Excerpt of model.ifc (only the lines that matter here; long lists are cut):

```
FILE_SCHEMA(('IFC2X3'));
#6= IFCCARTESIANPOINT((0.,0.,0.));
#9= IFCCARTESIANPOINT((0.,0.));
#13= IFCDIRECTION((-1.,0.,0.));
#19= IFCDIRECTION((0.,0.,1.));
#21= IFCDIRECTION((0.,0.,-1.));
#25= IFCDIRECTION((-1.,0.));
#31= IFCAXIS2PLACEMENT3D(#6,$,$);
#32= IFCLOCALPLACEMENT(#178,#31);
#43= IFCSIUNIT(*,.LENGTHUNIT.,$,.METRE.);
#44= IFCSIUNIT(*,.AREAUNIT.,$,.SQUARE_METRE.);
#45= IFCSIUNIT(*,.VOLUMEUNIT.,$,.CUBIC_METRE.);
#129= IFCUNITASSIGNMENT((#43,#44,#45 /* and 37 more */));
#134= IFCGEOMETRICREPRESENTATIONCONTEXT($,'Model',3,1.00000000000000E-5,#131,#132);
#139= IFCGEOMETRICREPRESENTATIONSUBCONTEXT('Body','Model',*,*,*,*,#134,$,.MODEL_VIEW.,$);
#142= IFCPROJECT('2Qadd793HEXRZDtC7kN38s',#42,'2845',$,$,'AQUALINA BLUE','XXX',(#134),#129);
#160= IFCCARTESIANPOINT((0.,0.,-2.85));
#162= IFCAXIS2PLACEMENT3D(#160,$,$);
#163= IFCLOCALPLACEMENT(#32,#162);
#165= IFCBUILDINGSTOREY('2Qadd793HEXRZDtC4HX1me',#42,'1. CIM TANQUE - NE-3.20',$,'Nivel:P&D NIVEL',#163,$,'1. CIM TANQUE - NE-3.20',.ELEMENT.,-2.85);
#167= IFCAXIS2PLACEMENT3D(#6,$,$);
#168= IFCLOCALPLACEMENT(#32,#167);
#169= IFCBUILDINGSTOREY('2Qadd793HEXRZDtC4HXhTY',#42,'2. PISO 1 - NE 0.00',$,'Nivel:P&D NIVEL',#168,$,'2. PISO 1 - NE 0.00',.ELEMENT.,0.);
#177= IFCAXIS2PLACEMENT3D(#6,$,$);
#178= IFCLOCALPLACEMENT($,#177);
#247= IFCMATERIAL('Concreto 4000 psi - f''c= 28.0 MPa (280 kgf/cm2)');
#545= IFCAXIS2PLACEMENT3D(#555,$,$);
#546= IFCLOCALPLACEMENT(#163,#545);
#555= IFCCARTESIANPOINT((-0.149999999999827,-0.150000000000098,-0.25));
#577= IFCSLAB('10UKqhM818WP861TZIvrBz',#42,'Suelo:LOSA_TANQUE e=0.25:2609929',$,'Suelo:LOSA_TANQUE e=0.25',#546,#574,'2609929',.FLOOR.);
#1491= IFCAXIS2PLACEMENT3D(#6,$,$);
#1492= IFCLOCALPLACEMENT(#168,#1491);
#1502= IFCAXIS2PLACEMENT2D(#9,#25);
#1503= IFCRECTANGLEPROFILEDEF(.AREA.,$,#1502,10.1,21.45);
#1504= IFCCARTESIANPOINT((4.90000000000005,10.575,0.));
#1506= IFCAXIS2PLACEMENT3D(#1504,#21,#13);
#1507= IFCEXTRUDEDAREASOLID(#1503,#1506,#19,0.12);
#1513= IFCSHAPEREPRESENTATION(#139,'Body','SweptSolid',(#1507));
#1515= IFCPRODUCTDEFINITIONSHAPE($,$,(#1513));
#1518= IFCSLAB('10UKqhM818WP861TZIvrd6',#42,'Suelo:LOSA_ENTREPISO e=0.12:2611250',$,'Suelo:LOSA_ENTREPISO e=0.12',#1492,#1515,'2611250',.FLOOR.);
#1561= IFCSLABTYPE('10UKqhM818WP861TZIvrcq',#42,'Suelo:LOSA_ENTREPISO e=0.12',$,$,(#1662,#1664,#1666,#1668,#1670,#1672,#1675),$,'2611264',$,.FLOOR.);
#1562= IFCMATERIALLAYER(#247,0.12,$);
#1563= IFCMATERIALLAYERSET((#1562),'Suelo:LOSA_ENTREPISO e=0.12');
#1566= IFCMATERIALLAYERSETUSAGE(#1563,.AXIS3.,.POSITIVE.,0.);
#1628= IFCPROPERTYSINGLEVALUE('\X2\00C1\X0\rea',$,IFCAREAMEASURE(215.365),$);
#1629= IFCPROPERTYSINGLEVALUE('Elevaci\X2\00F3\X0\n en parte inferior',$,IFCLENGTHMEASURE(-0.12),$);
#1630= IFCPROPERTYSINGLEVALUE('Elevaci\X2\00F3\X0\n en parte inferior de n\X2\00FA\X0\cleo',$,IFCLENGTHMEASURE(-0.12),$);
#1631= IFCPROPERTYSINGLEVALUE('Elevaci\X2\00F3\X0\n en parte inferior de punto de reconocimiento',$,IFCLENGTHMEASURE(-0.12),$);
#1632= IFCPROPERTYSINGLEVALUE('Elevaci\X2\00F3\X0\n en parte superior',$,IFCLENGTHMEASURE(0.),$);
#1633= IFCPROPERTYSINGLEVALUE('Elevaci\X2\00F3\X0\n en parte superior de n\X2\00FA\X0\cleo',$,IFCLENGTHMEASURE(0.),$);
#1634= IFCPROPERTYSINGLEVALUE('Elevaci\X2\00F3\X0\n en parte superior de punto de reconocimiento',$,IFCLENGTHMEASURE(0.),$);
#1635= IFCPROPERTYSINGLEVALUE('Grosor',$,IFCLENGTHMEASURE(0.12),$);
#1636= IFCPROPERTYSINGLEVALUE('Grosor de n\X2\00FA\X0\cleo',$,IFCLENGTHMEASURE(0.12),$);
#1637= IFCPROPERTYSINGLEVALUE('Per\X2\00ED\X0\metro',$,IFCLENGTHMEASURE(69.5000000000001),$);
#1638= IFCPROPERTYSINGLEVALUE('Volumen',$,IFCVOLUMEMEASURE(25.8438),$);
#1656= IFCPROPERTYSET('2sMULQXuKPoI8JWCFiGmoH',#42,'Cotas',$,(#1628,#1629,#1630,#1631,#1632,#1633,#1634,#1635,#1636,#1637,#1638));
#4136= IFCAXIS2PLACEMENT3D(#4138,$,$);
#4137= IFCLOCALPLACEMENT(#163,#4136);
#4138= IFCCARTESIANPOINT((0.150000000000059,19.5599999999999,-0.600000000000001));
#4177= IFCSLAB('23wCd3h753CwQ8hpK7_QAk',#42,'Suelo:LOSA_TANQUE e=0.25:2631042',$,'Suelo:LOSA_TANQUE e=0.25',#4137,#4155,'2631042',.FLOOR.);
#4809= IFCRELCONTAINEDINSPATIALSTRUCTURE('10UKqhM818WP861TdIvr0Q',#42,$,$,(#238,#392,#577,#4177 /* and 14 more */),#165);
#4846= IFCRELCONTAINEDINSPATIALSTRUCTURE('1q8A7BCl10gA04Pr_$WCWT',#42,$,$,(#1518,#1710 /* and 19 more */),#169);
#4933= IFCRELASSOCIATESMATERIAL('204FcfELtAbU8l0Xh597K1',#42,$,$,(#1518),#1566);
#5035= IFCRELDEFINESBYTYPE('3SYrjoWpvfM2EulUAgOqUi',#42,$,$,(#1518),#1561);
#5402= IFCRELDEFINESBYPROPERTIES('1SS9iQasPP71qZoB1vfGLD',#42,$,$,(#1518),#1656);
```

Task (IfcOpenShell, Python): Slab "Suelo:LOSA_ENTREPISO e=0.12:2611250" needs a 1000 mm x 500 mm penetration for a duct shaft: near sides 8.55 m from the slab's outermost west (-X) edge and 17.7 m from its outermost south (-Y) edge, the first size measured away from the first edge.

```python
import numpy as np
import ifcopenshell
import ifcopenshell.api.feature
import ifcopenshell.api.geometry
import ifcopenshell.api.pset
import ifcopenshell.api.root
import ifcopenshell.geom
import ifcopenshell.util.element
import ifcopenshell.util.placement
import ifcopenshell.util.representation
import ifcopenshell.util.shape
import ifcopenshell.util.unit

model = ifcopenshell.open("model.ifc")
unit_scale = ifcopenshell.util.unit.calculate_unit_scale(model)
area_scale = ifcopenshell.util.unit.calculate_unit_scale(model, "AREAUNIT")
volume_scale = ifcopenshell.util.unit.calculate_unit_scale(model, "VOLUMEUNIT")
settings = ifcopenshell.geom.settings()


def volume(element):
    """Net volume in cubic metres, openings subtracted."""
    shape = ifcopenshell.geom.create_shape(settings, element)
    return ifcopenshell.util.shape.get_volume(shape.geometry)


slab = model.by_id(1518)
before = volume(slab)

# Extent in the slab's own axes, in metres. The edges named are its -X and -Y sides.
slab_shape = ifcopenshell.geom.create_shape(settings, slab)
vertices = ifcopenshell.util.shape.get_vertices(slab_shape.geometry)
x_min, y_min, bottom = vertices.min(axis=0)
top = vertices[:, 2].max()

opening = ifcopenshell.api.root.create_entity(model, ifc_class="IfcOpeningElement", name="Duct shaft opening")
context = ifcopenshell.util.representation.get_context(model, "Model", "Body", "MODEL_VIEW")
width, depth = 1, 0.5
outline = [(0.0, 0.0), (width, 0.0), (width, depth), (0.0, depth), (0.0, 0.0)]
# Overshoot both faces by 50 mm so the cut is clean.
shape = ifcopenshell.api.geometry.add_slab_representation(
    model, context=context, depth=top - bottom + 0.1, polyline=outline
)
ifcopenshell.api.geometry.assign_representation(model, product=opening, representation=shape)

matrix = ifcopenshell.util.placement.get_local_placement(slab.ObjectPlacement)
matrix[:, 3] = matrix @ np.append(np.array([x_min + 8.55, y_min + 17.7, bottom - 0.05]) / unit_scale, 1.0)
ifcopenshell.api.geometry.edit_object_placement(model, product=opening, matrix=matrix, is_si=False)
ifcopenshell.api.feature.add_feature(model, feature=opening, element=slab)

after = volume(slab)

# Update the slab's stored quantities.
pset = model.by_id(ifcopenshell.util.element.get_pset(slab, "Cotas", should_inherit=False)["id"])
ifcopenshell.api.pset.edit_pset(model, pset=pset, properties={
    "Área": model.create_entity("IfcAreaMeasure", after / (top - bottom) / area_scale),
    "Volumen": model.create_entity("IfcVolumeMeasure", after / volume_scale),
})

print(f"slab volume {before:.3f} -> {after:.3f} m3")

model.write("model_v2.ifc")
```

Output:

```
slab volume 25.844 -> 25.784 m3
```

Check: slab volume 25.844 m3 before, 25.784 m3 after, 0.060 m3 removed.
